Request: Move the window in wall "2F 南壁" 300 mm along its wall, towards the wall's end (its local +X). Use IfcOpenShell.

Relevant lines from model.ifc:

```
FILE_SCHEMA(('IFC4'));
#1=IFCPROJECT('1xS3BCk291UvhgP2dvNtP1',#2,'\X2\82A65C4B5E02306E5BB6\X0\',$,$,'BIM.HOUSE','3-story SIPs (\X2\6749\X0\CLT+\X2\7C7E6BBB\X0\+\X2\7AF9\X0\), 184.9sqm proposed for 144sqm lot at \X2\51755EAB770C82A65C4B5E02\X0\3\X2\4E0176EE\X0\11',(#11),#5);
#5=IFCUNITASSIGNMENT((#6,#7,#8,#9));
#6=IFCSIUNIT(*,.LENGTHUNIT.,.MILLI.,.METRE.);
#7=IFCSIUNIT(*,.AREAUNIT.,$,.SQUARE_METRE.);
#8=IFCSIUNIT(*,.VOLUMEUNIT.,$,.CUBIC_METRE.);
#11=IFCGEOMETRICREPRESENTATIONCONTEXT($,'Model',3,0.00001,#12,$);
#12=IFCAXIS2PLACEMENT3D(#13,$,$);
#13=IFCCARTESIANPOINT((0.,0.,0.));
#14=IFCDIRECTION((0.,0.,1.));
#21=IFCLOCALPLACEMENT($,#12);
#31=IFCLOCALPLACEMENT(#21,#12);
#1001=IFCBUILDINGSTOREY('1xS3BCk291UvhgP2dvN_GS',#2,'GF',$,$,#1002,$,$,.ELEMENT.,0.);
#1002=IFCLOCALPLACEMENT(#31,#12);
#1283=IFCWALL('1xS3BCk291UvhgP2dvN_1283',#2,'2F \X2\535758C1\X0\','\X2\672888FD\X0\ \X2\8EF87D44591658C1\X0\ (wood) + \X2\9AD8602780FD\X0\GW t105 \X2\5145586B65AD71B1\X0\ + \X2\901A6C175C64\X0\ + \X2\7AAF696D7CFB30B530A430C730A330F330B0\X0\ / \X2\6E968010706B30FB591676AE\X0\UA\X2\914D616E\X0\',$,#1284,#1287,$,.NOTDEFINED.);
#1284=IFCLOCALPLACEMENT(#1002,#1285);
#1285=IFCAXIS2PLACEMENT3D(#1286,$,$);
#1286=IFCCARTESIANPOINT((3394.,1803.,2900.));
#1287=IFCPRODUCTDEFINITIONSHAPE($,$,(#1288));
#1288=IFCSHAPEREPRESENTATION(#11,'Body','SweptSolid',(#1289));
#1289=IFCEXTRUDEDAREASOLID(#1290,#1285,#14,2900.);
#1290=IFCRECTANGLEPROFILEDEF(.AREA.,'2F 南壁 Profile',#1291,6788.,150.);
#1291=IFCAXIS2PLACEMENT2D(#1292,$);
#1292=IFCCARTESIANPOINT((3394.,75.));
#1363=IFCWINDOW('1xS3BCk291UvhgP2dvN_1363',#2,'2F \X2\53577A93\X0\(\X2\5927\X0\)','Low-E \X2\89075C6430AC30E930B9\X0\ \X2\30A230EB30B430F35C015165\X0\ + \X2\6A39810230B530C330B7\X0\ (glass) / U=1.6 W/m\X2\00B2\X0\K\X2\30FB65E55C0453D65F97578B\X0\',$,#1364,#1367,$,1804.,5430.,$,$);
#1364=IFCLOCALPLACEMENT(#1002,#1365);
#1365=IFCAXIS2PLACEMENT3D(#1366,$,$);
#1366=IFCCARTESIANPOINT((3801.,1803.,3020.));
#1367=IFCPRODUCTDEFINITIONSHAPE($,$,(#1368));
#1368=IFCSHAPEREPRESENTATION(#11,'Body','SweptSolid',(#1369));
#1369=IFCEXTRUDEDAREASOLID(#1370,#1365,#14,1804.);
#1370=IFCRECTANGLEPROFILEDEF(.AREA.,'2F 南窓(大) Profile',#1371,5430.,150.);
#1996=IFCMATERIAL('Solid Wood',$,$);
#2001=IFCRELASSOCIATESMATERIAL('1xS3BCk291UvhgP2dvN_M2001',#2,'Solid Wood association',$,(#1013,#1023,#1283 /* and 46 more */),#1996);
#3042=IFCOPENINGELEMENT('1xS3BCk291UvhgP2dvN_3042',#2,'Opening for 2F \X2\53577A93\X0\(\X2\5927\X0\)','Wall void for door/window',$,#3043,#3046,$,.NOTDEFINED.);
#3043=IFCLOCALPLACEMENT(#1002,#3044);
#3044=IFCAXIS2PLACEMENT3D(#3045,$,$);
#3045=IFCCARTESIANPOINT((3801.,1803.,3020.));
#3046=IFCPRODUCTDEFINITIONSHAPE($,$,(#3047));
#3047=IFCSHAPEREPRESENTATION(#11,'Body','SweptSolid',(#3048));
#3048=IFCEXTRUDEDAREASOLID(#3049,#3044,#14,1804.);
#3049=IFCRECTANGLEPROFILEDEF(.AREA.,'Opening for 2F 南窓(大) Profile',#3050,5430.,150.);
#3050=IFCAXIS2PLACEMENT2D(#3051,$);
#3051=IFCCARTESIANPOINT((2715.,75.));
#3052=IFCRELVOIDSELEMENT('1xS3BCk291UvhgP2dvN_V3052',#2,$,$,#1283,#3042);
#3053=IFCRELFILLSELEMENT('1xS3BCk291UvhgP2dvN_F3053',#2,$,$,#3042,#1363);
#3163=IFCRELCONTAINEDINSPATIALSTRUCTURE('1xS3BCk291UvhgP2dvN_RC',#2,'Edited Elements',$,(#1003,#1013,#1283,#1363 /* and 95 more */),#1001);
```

```python
import ifcopenshell
import ifcopenshell.api.geometry
import ifcopenshell.util.placement
import ifcopenshell.util.unit

model = ifcopenshell.open("model.ifc")
unit_scale = ifcopenshell.util.unit.calculate_unit_scale(model)

window = model.by_id(1363)
opening = window.FillsVoids[0].RelatingOpeningElement
wall = opening.VoidsElements[0].RelatingBuildingElement

wall_matrix = ifcopenshell.util.placement.get_local_placement(wall.ObjectPlacement)
shift = wall_matrix[:3, 0] * 0.3 / unit_scale
before = ifcopenshell.util.placement.get_local_placement(window.ObjectPlacement)[:3, 3].copy()

# The window is not placed relative to its opening, so move both.
for product in (opening, window):
    matrix = ifcopenshell.util.placement.get_local_placement(product.ObjectPlacement)
    matrix[:3, 3] += shift
    ifcopenshell.api.geometry.edit_object_placement(model, product=product, matrix=matrix, is_si=False)

after = ifcopenshell.util.placement.get_local_placement(window.ObjectPlacement)[:3, 3]
print("window moved by", (after - before).round(3) + 0.0)

model.write("model_edited.ifc")
```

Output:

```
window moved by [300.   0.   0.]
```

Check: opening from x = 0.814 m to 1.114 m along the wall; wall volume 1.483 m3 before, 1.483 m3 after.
